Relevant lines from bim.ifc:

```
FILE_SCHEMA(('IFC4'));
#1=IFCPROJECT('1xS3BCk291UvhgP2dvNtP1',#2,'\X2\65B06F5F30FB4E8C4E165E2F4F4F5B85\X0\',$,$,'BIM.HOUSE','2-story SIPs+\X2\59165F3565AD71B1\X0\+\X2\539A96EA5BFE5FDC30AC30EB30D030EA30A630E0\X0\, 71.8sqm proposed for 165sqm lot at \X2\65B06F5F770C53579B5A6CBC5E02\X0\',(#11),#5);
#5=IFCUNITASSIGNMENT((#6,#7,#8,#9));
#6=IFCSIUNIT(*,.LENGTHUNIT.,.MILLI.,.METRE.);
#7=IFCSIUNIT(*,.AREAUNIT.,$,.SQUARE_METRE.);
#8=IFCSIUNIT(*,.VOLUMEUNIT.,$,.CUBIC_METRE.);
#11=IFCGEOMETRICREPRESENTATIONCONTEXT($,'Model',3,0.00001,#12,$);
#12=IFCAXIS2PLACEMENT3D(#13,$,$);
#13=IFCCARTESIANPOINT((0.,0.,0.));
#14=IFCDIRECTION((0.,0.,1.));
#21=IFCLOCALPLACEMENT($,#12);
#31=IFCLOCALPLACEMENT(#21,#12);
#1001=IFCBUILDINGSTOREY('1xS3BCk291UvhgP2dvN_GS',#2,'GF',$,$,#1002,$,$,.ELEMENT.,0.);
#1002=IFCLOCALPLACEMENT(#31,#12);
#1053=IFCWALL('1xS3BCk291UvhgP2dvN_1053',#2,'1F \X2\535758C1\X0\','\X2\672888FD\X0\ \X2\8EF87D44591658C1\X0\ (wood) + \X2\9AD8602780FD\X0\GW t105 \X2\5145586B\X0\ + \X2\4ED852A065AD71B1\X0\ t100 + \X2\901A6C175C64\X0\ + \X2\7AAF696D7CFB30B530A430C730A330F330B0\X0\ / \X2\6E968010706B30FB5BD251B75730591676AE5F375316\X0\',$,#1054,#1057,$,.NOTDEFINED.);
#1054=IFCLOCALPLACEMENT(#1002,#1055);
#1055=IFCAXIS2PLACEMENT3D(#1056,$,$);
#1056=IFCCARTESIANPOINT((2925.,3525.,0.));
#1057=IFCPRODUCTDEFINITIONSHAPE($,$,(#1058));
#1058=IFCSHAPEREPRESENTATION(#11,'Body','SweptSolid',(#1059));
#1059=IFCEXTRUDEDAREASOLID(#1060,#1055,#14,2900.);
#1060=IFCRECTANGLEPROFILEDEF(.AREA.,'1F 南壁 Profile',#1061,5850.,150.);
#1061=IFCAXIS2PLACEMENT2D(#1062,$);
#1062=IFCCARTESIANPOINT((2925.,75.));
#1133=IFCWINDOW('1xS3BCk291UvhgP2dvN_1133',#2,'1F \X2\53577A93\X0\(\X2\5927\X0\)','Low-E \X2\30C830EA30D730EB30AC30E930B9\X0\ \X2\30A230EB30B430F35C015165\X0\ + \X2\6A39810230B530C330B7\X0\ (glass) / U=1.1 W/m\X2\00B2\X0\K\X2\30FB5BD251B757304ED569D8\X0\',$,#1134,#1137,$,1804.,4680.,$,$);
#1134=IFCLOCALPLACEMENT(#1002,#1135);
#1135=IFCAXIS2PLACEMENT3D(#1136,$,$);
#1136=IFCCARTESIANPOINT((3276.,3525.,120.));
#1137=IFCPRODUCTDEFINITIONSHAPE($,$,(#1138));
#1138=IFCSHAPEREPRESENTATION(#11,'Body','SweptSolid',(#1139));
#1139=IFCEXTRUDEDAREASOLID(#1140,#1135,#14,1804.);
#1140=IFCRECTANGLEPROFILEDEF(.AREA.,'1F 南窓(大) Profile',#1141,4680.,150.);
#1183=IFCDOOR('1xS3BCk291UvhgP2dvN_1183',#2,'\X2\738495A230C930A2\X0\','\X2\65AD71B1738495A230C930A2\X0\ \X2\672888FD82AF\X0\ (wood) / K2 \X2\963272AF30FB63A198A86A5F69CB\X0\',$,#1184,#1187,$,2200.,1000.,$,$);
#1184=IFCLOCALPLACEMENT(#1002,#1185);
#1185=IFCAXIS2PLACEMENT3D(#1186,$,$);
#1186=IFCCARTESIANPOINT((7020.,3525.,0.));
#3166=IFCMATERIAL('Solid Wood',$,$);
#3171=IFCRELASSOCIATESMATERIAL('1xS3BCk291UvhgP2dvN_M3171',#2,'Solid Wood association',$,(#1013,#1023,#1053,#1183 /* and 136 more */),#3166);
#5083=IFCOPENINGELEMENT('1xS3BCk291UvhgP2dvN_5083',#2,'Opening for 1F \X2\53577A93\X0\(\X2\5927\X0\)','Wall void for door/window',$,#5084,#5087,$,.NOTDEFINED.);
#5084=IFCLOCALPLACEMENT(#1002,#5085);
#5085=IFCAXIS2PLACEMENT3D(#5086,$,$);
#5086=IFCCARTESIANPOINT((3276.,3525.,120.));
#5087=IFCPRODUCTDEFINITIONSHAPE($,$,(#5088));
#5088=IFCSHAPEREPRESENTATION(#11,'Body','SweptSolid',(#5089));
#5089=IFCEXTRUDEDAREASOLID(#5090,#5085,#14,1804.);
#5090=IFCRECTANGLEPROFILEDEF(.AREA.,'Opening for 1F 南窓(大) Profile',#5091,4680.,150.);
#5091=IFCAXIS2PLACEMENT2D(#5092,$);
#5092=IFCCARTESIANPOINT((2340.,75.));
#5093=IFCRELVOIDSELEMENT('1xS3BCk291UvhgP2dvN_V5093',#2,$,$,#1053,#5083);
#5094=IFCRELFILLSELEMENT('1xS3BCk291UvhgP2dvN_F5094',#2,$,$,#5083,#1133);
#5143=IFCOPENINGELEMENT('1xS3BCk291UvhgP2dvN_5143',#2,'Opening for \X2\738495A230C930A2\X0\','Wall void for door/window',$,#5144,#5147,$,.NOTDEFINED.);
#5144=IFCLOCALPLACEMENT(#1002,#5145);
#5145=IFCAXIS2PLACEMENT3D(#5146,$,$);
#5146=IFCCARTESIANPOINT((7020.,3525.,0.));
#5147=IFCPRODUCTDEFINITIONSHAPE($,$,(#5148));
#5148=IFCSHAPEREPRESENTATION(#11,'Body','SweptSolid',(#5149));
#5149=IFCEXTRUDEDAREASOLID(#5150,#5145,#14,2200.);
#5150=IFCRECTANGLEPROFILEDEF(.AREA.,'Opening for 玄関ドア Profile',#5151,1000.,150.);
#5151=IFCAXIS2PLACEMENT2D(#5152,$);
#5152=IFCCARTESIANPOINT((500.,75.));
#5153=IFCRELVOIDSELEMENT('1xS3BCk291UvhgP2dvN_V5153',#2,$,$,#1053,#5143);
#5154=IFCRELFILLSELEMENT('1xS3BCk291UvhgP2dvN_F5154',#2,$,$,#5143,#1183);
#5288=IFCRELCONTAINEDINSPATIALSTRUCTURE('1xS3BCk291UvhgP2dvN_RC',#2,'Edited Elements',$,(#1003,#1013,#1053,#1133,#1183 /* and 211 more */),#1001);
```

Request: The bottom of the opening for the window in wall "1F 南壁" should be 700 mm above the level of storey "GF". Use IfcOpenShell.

```python
import numpy as np
import ifcopenshell
import ifcopenshell.api.geometry
import ifcopenshell.geom
import ifcopenshell.util.element
import ifcopenshell.util.placement
import ifcopenshell.util.shape
import ifcopenshell.util.unit

model = ifcopenshell.open("bim.ifc")
unit_scale = ifcopenshell.util.unit.calculate_unit_scale(model)

window = model.by_guid("1xS3BCk291UvhgP2dvN_1133")
opening = window.FillsVoids[0].RelatingOpeningElement
storey = ifcopenshell.util.element.get_container(window, ifc_class="IfcBuildingStorey")
level = ifcopenshell.util.placement.get_local_placement(storey.ObjectPlacement)[2, 3]

# The opening's origin need not be at the sill, so measure its lowest point.
shape = ifcopenshell.geom.create_shape(ifcopenshell.geom.settings(), opening)
bottom = ifcopenshell.util.shape.get_shape_bottom_elevation(shape, shape.geometry) / unit_scale
dz = level + 0.7 / unit_scale - bottom

shift = np.array([0.0, 0.0, dz])
# The window is not placed relative to its opening, so move both.
for product in (opening, window):
    matrix = ifcopenshell.util.placement.get_local_placement(product.ObjectPlacement)
    matrix[:3, 3] += shift
    ifcopenshell.api.geometry.edit_object_placement(model, product=product, matrix=matrix, is_si=False)

print(f"moved by {dz * unit_scale:+.3f} m")

model.write("bim_v2.ifc")
```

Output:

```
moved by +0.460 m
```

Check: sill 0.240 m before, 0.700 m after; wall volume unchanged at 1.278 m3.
